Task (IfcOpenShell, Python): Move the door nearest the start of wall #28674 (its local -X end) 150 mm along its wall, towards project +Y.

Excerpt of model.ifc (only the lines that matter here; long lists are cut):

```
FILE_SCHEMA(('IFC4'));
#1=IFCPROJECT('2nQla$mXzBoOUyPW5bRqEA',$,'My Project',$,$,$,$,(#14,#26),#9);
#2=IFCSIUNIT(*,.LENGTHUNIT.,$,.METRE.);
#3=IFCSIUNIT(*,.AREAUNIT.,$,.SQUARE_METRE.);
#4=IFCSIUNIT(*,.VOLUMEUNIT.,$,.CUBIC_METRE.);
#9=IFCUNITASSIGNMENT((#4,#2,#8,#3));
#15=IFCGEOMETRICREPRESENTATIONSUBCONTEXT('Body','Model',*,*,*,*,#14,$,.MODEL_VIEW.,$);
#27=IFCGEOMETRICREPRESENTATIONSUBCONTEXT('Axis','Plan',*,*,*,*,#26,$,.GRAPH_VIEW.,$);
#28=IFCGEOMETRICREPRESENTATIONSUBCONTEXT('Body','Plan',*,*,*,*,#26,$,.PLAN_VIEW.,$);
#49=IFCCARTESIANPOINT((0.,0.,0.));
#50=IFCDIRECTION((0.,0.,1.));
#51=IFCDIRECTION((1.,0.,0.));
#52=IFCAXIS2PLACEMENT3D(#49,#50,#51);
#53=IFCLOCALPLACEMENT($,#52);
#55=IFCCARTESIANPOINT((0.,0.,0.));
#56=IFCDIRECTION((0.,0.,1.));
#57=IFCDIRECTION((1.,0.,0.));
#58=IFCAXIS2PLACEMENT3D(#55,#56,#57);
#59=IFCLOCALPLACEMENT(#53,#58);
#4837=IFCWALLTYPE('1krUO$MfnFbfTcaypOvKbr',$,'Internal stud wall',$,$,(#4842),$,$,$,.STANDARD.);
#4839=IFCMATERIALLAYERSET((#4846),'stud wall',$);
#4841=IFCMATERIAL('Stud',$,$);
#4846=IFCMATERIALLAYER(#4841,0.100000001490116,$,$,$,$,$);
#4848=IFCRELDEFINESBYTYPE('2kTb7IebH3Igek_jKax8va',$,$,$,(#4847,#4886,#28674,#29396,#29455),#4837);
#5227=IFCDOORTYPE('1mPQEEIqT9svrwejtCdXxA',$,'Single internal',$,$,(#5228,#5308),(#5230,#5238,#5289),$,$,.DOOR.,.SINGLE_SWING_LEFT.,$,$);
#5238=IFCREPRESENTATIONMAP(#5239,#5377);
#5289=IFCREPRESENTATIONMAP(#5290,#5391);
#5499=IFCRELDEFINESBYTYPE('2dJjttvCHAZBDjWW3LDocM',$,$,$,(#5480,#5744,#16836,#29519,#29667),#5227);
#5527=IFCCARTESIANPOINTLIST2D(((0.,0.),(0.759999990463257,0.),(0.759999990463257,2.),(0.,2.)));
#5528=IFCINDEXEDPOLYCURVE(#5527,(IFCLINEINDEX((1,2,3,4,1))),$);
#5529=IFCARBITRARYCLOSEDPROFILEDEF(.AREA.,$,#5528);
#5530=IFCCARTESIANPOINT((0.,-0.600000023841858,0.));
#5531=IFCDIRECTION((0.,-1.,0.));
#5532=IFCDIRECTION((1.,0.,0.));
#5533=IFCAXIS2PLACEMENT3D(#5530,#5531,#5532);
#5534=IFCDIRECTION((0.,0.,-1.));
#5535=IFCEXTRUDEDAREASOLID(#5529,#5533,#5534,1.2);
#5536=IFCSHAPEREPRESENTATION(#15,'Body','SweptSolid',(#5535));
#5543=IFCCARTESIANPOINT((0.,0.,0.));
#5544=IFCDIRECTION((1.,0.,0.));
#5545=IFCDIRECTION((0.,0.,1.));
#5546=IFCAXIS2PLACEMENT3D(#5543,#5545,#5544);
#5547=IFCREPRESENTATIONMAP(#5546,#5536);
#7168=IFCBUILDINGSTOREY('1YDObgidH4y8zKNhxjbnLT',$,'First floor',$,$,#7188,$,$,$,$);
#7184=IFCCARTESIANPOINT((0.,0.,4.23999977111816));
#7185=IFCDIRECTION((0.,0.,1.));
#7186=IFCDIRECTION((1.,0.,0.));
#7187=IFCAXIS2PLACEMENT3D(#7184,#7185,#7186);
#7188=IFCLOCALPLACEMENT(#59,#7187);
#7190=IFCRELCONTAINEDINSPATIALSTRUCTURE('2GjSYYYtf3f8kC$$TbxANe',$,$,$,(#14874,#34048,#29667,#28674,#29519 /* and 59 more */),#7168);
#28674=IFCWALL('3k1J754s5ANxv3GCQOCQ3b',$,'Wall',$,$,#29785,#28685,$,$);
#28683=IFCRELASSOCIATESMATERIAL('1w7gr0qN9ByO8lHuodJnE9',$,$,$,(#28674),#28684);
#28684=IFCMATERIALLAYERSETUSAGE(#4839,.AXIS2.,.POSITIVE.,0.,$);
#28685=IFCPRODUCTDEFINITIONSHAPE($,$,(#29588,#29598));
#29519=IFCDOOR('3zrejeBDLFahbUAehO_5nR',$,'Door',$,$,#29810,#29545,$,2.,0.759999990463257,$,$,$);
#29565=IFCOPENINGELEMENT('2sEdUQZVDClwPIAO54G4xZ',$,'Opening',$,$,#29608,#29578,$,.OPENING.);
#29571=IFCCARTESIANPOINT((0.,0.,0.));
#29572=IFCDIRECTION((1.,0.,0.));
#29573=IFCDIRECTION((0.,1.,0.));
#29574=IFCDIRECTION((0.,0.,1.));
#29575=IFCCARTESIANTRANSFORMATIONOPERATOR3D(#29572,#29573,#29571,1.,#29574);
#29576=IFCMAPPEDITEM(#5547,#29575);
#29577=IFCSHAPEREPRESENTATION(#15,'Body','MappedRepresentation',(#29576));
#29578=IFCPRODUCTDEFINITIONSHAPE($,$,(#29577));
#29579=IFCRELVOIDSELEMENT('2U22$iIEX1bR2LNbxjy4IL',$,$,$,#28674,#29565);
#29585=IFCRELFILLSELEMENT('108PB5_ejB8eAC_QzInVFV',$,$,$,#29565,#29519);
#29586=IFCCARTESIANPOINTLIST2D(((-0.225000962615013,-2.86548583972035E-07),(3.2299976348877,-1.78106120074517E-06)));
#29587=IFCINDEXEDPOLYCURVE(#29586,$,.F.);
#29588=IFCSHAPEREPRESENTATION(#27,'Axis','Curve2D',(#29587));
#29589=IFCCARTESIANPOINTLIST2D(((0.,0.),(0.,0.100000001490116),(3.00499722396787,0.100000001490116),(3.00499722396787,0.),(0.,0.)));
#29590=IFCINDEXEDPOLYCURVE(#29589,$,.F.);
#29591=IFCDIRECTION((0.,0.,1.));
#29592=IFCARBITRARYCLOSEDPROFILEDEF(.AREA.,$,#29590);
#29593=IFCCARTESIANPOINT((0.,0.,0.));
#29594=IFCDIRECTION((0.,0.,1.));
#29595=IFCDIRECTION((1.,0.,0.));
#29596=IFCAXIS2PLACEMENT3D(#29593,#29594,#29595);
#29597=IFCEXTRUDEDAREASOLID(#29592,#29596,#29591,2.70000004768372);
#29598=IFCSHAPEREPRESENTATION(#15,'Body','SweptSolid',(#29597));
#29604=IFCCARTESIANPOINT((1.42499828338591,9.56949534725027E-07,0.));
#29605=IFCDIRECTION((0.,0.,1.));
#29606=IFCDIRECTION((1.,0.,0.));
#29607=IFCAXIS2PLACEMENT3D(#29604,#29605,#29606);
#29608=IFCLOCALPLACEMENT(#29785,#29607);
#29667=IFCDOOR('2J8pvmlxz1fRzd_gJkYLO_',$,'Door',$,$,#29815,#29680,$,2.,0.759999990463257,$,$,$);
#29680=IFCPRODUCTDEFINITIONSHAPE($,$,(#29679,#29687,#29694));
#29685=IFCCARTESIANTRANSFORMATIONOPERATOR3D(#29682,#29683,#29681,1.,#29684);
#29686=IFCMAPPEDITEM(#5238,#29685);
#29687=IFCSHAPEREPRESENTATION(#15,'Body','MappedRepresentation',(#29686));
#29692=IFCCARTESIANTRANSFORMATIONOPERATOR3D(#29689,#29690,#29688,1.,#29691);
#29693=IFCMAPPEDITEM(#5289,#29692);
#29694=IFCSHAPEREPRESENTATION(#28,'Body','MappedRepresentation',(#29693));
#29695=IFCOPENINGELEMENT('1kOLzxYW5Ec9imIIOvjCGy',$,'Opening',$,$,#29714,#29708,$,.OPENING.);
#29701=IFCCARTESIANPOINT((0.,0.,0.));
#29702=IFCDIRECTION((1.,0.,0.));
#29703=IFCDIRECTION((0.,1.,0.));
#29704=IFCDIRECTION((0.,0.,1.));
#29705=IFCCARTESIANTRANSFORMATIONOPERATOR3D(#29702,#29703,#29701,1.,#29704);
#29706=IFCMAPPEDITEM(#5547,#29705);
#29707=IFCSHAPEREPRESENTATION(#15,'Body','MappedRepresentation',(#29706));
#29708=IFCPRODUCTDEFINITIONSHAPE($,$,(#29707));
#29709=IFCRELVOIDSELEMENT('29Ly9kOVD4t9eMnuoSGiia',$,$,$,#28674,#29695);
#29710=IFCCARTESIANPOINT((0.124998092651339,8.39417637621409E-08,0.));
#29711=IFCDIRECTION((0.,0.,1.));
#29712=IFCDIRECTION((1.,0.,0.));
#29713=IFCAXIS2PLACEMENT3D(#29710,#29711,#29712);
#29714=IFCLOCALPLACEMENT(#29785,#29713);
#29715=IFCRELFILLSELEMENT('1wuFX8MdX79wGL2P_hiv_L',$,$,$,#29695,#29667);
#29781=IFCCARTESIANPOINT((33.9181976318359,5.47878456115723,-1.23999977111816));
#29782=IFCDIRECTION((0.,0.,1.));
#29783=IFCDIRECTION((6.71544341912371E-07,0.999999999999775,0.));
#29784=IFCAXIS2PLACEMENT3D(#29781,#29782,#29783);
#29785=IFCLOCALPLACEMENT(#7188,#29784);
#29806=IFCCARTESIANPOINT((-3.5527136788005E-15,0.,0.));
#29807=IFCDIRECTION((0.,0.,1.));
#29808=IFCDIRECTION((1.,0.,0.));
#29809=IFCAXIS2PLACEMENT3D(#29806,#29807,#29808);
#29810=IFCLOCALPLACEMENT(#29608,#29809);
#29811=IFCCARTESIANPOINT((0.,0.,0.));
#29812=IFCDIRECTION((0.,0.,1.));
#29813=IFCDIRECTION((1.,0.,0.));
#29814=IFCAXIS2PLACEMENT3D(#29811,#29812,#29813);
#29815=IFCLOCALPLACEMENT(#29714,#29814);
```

```python
import ifcopenshell
import ifcopenshell.api.geometry
import ifcopenshell.util.placement

model = ifcopenshell.open("model.ifc")

door = model.by_guid("2J8pvmlxz1fRzd_gJkYLO_")
opening = door.FillsVoids[0].RelatingOpeningElement
wall = opening.VoidsElements[0].RelatingBuildingElement

wall_matrix = ifcopenshell.util.placement.get_local_placement(wall.ObjectPlacement)
shift = wall_matrix[:3, 0] * 0.15
before = ifcopenshell.util.placement.get_local_placement(door.ObjectPlacement)[:3, 3].copy()

# The door is placed relative to its opening, so it follows when the opening moves.
matrix = ifcopenshell.util.placement.get_local_placement(opening.ObjectPlacement)
matrix[:3, 3] += shift
ifcopenshell.api.geometry.edit_object_placement(
    model, product=opening, matrix=matrix, is_si=False, should_transform_children=True
)

after = ifcopenshell.util.placement.get_local_placement(door.ObjectPlacement)[:3, 3]
print("door moved by", (after - before).round(3) + 0.0)

model.write("model_v2.ifc")
```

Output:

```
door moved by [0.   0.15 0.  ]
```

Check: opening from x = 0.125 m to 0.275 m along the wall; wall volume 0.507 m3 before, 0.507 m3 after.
